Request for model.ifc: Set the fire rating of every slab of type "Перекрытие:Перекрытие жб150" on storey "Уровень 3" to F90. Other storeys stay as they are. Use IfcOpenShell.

First a look at what the model holds.

```python
import ifcopenshell
import ifcopenshell.util.element

model = ifcopenshell.open("model.ifc")
print(model.schema)
storey = next(s for s in model.by_type("IfcBuildingStorey") if s.Name == "Уровень 3")
slabs = [e for e in ifcopenshell.util.element.get_decomposition(storey) if e.is_a("IfcSlab")]
seen = {}
for e in slabs:
    element_type = ifcopenshell.util.element.get_type(e)
    key = (element_type.Name if element_type != e and element_type else None, ifcopenshell.util.element.get_pset(e, "Pset_SlabCommon", "FireRating"))
    seen[key] = seen.get(key, 0) + 1
for (name, value), count in sorted(seen.items(), key=str):
    print(count, "x", name, "|", value)
```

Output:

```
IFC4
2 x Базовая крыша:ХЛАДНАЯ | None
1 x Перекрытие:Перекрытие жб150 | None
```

```python
import ifcopenshell
import ifcopenshell.api.pset
import ifcopenshell.util.element

model = ifcopenshell.open("model.ifc")

storey = next(s for s in model.by_type("IfcBuildingStorey") if s.Name == "Уровень 3")
slabs = [e for e in ifcopenshell.util.element.get_decomposition(storey) if e.is_a("IfcSlab")]

count = 0
for e in slabs:
    element_type = ifcopenshell.util.element.get_type(e)
    if element_type in (None, e) or element_type.Name != "Перекрытие:Перекрытие жб150":
        continue
    # add_pset returns the element's existing set when there is one.
    pset = ifcopenshell.api.pset.add_pset(model, product=e, name="Pset_SlabCommon")
    ifcopenshell.api.pset.edit_pset(model, pset=pset, properties={"FireRating": "F90"})
    count += 1

print(count, "slabs updated")

model.write("model_rev.ifc")
```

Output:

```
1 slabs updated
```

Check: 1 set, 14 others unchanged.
